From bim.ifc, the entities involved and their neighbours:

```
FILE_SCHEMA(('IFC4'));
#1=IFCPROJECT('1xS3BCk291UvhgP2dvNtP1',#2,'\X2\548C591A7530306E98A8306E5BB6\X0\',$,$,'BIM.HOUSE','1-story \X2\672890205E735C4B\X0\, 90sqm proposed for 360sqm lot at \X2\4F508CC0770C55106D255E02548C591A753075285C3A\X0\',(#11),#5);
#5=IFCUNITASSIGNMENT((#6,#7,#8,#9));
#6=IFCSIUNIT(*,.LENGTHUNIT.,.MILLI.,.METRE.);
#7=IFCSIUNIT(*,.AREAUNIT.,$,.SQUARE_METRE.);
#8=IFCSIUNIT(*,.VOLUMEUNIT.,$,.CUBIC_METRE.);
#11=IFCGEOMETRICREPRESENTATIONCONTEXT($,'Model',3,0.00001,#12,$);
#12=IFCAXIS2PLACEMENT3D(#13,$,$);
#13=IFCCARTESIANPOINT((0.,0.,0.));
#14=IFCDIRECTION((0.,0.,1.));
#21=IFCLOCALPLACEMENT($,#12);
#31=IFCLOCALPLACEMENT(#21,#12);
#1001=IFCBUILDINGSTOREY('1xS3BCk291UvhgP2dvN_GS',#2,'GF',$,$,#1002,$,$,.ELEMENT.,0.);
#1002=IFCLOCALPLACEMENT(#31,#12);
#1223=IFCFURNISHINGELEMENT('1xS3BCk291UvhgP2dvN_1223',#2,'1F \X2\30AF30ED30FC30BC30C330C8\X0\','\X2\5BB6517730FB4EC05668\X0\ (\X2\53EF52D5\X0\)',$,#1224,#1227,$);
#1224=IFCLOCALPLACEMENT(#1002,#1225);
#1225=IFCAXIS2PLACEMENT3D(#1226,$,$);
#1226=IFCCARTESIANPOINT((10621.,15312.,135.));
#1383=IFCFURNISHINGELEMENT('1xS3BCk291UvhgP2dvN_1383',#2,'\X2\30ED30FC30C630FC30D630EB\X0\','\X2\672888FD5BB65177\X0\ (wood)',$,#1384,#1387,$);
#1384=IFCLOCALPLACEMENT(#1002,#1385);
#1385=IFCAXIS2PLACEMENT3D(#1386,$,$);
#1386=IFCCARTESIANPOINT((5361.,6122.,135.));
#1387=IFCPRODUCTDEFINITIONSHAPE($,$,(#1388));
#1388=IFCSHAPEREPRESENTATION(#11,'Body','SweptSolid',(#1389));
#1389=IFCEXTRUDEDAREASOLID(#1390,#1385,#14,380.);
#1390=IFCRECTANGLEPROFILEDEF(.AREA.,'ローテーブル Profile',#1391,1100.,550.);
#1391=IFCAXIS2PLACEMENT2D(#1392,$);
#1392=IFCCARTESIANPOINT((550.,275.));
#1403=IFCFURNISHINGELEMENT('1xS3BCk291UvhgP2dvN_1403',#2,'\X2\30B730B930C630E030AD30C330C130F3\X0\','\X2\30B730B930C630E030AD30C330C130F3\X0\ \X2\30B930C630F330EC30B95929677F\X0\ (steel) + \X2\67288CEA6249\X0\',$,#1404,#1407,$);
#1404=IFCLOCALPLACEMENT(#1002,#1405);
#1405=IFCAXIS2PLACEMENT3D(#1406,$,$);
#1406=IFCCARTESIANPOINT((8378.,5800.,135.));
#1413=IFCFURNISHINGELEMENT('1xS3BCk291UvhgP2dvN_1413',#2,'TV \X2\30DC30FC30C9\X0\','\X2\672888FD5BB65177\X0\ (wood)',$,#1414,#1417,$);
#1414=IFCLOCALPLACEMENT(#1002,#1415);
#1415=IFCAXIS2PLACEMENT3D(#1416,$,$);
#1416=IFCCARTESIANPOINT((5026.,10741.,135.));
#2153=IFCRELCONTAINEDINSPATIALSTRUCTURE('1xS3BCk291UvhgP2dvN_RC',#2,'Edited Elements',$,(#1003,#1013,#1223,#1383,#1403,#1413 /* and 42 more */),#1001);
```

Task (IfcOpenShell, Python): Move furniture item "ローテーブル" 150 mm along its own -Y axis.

```python
import ifcopenshell
import ifcopenshell.api.geometry
import ifcopenshell.util.placement
import ifcopenshell.util.unit

model = ifcopenshell.open("bim.ifc")
unit_scale = ifcopenshell.util.unit.calculate_unit_scale(model)

item = model.by_guid("1xS3BCk291UvhgP2dvN_1383")
matrix = ifcopenshell.util.placement.get_local_placement(item.ObjectPlacement)
matrix[:3, 3] -= matrix[:3, 1] * 0.15 / unit_scale
ifcopenshell.api.geometry.edit_object_placement(model, product=item, matrix=matrix, is_si=False)

print(ifcopenshell.util.placement.get_local_placement(item.ObjectPlacement).round(3) + 0.0)

model.write("bim_edited.ifc")
```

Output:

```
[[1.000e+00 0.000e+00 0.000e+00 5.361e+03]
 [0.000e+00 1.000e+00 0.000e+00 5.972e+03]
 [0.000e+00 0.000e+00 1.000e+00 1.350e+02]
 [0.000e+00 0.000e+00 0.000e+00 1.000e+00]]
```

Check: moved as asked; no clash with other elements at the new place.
